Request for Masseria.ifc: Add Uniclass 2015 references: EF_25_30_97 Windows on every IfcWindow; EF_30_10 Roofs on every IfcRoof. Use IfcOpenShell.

First a look at what the model holds.

```python
import ifcopenshell

model = ifcopenshell.open("Masseria.ifc")
print(model.schema)
print("classifications:", [c.Name for c in model.by_type("IfcClassification")])
for ifc_class in ("IfcDoor", "IfcRoof", "IfcStair", "IfcWall", "IfcWindow"):
    print(ifc_class, len(model.by_type(ifc_class)))
```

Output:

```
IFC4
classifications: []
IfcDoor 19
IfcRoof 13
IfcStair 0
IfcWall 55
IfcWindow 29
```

```python
import ifcopenshell
import ifcopenshell.api.classification

model = ifcopenshell.open("Masseria.ifc")

system = ifcopenshell.api.classification.add_classification(model, classification="Uniclass 2015")

codes = {
    "IfcWindow": ("EF_25_30_97", "Windows"),
    "IfcRoof": ("EF_30_10", "Roofs"),
}
for ifc_class, (code, name) in codes.items():
    products = model.by_type(ifc_class)
    ifcopenshell.api.classification.add_reference(
        model, products=products, classification=system, identification=code, name=name
    )
    print(code, len(products))

model.write("Masseria_edited.ifc")
```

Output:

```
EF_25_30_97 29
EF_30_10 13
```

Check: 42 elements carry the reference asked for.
